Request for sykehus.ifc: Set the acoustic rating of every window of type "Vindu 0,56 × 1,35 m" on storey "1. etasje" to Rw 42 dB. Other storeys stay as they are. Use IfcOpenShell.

First a look at what the model holds.

```python
import ifcopenshell
import ifcopenshell.util.element

model = ifcopenshell.open("sykehus.ifc")
print(model.schema)
storey = next(s for s in model.by_type("IfcBuildingStorey") if s.Name == "1. etasje")
windows = [e for e in ifcopenshell.util.element.get_decomposition(storey) if e.is_a("IfcWindow")]
seen = {}
for e in windows:
    element_type = ifcopenshell.util.element.get_type(e)
    key = (element_type.Name if element_type != e and element_type else None, ifcopenshell.util.element.get_pset(e, "Pset_WindowCommon", "AcousticRating"))
    seen[key] = seen.get(key, 0) + 1
for (name, value), count in sorted(seen.items(), key=str):
    print(count, "x", name, "|", value)
```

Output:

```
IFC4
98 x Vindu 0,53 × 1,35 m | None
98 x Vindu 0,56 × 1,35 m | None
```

```python
import ifcopenshell
import ifcopenshell.api.pset
import ifcopenshell.util.element

model = ifcopenshell.open("sykehus.ifc")

storey = next(s for s in model.by_type("IfcBuildingStorey") if s.Name == "1. etasje")
windows = [e for e in ifcopenshell.util.element.get_decomposition(storey) if e.is_a("IfcWindow")]

count = 0
for e in windows:
    element_type = ifcopenshell.util.element.get_type(e)
    if element_type in (None, e) or element_type.Name != "Vindu 0,56 × 1,35 m":
        continue
    found = ifcopenshell.util.element.get_pset(e, "Pset_WindowCommon", should_inherit=False)
    if found:
        pset = model.by_id(found["id"])
        if len(ifcopenshell.util.element.get_elements_by_pset(pset)) > 1:
            pset = ifcopenshell.api.pset.unshare_pset(model, products=[e], pset=pset)[0]
    else:
        pset = ifcopenshell.api.pset.add_pset(model, product=e, name="Pset_WindowCommon")
    ifcopenshell.api.pset.edit_pset(model, pset=pset, properties={"AcousticRating": "Rw 42 dB"})
    count += 1

print(count, "windows updated")

model.write("sykehus_updated.ifc")
```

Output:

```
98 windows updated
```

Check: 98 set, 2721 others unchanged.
